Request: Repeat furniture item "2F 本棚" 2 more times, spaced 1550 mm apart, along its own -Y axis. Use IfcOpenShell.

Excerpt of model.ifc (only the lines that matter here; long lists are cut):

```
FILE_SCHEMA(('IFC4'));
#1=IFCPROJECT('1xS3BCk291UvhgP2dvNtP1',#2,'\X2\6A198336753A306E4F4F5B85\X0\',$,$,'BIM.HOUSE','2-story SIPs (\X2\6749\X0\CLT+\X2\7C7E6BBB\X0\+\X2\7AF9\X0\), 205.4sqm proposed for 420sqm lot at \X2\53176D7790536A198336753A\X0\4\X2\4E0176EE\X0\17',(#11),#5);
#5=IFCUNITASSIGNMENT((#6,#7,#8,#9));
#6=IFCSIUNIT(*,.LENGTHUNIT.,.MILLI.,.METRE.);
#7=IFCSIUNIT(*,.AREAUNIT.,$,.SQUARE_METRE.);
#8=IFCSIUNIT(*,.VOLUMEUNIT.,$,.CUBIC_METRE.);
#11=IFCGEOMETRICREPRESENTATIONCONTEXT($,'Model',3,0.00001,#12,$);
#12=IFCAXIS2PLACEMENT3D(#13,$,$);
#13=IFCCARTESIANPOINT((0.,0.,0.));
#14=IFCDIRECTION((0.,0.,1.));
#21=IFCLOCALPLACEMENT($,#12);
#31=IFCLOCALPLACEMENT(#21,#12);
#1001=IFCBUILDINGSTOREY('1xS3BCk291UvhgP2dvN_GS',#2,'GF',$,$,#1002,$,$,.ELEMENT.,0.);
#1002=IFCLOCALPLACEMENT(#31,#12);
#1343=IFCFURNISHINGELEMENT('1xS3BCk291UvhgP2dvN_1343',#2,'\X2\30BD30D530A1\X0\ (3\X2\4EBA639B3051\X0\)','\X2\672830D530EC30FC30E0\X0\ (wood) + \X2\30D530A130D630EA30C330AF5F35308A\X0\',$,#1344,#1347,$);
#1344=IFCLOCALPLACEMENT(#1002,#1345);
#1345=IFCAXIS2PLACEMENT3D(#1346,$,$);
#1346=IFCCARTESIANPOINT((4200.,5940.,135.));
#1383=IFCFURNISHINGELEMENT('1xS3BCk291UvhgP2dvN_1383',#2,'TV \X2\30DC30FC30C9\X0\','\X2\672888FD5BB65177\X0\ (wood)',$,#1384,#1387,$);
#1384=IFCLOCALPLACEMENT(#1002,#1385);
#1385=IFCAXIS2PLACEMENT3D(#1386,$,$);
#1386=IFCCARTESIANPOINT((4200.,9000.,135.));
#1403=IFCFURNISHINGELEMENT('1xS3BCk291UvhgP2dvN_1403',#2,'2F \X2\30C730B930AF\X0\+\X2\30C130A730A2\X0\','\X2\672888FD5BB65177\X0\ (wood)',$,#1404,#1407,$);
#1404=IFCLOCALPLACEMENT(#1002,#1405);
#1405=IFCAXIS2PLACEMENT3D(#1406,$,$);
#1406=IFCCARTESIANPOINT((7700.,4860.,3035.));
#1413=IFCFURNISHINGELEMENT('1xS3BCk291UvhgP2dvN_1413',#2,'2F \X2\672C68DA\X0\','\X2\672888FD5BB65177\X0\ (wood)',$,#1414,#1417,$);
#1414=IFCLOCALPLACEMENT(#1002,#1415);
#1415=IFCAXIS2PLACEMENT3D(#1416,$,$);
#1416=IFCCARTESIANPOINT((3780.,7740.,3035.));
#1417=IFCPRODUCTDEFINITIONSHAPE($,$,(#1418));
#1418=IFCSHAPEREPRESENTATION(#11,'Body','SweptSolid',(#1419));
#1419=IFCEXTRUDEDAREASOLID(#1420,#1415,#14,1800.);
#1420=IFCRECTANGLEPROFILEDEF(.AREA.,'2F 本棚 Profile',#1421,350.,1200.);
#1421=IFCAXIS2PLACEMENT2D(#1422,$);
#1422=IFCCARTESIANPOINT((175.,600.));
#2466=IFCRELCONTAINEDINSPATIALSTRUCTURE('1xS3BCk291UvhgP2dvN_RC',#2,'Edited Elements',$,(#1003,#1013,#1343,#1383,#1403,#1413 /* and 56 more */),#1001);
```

```python
import ifcopenshell
import ifcopenshell.api.geometry
import ifcopenshell.api.root
import ifcopenshell.util.element
import ifcopenshell.util.placement

model = ifcopenshell.open("model.ifc")


def reuse_history(source, copy):
    """copy_class also copies each property set's owner history, people and application; keep the originals."""
    for rel in copy.IsDefinedBy:
        if rel.is_a("IfcRelDefinesByProperties") and (history := rel.RelatingPropertyDefinition.OwnerHistory):
            rel.RelatingPropertyDefinition.OwnerHistory = source.OwnerHistory
            ifcopenshell.util.element.remove_deep2(model, history)


source = model.by_guid("1xS3BCk291UvhgP2dvN_1413")
base = ifcopenshell.util.placement.get_local_placement(source.ObjectPlacement)
step = -base[:3, 1] * 1550.0

for i in range(1, 3):
    copy = ifcopenshell.api.root.copy_class(model, product=source)
    copy.Representation = ifcopenshell.util.element.copy_deep(
        model, source.Representation, exclude=["IfcGeometricRepresentationContext", "IfcRepresentationMap"]
    )
    reuse_history(source, copy)
    matrix = base.copy()
    matrix[:3, 3] += i * step
    print("added at", matrix[:3, 3].round(3) + 0.0)
    ifcopenshell.api.geometry.edit_object_placement(model, product=copy, matrix=matrix, is_si=False)

model.write("model_v2.ifc")
```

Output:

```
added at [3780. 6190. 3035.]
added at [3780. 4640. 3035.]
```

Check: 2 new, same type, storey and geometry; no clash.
